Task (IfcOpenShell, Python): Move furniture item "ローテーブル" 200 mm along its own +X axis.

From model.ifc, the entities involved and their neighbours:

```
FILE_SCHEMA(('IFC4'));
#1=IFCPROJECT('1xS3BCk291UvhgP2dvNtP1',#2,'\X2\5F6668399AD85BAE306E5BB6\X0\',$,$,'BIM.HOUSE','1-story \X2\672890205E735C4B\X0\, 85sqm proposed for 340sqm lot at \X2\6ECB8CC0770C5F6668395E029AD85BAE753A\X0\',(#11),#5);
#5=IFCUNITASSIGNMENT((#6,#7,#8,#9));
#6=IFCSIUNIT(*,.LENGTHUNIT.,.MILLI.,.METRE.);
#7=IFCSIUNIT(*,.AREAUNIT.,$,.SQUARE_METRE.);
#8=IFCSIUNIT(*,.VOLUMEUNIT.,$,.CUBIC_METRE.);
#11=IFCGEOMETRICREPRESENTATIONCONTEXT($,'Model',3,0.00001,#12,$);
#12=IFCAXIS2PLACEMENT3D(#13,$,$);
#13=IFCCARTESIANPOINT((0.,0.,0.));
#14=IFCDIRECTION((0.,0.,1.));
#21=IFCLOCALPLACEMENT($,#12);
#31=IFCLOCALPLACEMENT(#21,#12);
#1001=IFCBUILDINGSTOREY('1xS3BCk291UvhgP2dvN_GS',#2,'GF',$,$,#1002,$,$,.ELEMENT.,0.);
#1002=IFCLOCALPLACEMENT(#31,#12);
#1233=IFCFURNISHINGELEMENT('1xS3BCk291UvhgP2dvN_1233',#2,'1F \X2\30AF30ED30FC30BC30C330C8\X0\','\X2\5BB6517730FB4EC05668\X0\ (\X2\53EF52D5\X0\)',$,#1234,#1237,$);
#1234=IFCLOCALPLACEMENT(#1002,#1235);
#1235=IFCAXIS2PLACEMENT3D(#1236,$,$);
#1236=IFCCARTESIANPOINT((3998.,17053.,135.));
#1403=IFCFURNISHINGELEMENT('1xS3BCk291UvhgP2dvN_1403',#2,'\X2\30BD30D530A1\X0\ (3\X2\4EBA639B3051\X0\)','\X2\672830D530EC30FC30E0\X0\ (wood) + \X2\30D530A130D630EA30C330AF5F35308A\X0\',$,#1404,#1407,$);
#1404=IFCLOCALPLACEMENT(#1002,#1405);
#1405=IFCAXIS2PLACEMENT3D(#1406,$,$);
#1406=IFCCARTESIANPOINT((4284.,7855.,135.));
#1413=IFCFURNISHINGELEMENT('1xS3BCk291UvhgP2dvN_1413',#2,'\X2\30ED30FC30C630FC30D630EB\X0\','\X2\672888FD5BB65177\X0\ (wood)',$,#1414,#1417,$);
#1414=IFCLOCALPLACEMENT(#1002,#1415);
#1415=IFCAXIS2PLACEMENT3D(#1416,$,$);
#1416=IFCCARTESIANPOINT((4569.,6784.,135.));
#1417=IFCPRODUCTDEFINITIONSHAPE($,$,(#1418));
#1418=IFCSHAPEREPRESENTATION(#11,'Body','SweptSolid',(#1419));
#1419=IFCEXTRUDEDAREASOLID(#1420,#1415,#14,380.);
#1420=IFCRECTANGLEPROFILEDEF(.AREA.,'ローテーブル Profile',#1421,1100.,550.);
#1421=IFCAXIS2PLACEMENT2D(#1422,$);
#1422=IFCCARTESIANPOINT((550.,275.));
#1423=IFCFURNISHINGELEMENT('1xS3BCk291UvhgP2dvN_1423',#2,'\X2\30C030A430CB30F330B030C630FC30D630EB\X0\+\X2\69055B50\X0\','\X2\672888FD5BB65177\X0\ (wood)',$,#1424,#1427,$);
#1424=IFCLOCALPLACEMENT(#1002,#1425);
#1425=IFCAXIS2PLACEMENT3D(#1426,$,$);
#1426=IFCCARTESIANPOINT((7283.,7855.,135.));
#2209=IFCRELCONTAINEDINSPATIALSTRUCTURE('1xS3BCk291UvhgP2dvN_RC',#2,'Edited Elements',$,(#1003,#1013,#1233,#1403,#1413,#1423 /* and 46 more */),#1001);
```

```python
import ifcopenshell
import ifcopenshell.api.geometry
import ifcopenshell.util.placement
import ifcopenshell.util.unit

model = ifcopenshell.open("model.ifc")
unit_scale = ifcopenshell.util.unit.calculate_unit_scale(model)

item = model.by_guid("1xS3BCk291UvhgP2dvN_1413")
matrix = ifcopenshell.util.placement.get_local_placement(item.ObjectPlacement)
matrix[:3, 3] += matrix[:3, 0] * 0.2 / unit_scale
ifcopenshell.api.geometry.edit_object_placement(model, product=item, matrix=matrix, is_si=False)

print(ifcopenshell.util.placement.get_local_placement(item.ObjectPlacement).round(3) + 0.0)

model.write("model_edited.ifc")
```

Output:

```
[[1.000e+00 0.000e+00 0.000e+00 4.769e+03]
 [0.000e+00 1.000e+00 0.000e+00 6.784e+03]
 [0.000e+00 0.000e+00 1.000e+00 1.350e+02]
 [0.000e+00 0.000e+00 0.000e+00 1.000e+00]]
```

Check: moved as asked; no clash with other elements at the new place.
